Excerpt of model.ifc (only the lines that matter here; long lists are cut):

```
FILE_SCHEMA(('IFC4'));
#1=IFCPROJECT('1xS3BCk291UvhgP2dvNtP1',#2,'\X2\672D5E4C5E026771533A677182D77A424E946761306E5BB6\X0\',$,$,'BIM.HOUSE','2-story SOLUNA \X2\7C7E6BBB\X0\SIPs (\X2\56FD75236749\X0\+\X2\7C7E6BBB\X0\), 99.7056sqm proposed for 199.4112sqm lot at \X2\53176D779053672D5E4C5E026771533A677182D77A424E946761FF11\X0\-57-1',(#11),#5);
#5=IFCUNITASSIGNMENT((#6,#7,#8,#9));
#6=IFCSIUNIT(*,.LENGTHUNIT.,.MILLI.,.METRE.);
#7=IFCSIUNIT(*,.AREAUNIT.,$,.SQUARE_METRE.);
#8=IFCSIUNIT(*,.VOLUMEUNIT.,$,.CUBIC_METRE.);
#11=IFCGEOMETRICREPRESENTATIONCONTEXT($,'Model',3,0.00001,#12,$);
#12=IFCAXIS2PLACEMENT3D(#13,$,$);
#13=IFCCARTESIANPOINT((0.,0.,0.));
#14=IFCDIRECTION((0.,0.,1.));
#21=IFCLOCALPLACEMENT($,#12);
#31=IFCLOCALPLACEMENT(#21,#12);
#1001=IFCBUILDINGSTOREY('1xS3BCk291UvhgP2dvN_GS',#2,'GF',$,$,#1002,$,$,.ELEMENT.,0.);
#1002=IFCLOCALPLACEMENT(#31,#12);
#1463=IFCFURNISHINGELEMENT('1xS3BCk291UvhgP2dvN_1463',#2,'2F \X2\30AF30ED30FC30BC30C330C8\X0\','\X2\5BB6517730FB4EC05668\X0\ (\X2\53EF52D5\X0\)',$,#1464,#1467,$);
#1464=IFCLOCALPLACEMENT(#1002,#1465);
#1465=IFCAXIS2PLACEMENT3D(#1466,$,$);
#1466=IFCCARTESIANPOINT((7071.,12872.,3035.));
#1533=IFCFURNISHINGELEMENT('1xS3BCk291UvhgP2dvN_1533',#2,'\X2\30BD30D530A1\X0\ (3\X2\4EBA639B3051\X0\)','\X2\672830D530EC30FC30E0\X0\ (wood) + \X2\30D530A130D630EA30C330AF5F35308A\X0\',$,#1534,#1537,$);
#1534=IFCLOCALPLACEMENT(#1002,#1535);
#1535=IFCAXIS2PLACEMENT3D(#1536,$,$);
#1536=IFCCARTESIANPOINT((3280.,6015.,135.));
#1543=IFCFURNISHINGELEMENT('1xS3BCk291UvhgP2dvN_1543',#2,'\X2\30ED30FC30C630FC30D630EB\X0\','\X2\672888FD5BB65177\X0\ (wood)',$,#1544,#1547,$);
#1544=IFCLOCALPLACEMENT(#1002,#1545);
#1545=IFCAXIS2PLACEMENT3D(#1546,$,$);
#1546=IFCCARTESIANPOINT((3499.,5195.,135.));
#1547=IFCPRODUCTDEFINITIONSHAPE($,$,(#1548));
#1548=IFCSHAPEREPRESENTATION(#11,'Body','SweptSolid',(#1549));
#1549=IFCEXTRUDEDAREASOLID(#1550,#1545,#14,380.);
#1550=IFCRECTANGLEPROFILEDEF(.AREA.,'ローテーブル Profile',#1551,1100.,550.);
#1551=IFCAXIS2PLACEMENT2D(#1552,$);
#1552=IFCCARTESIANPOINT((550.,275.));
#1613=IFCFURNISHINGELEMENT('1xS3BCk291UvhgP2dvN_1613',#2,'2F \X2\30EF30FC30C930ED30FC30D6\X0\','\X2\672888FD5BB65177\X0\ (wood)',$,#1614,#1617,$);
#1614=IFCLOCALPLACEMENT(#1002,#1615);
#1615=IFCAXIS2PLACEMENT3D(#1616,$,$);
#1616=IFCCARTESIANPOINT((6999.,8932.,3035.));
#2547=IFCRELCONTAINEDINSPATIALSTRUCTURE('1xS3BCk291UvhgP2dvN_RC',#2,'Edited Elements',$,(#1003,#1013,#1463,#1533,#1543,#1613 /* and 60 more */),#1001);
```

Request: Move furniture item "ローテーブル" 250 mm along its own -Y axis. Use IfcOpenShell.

```python
import ifcopenshell
import ifcopenshell.api.geometry
import ifcopenshell.util.placement
import ifcopenshell.util.unit

model = ifcopenshell.open("model.ifc")
unit_scale = ifcopenshell.util.unit.calculate_unit_scale(model)

item = model.by_guid("1xS3BCk291UvhgP2dvN_1543")
matrix = ifcopenshell.util.placement.get_local_placement(item.ObjectPlacement)
matrix[:3, 3] -= matrix[:3, 1] * 0.25 / unit_scale
ifcopenshell.api.geometry.edit_object_placement(model, product=item, matrix=matrix, is_si=False)

print(ifcopenshell.util.placement.get_local_placement(item.ObjectPlacement).round(3) + 0.0)

model.write("model_updated.ifc")
```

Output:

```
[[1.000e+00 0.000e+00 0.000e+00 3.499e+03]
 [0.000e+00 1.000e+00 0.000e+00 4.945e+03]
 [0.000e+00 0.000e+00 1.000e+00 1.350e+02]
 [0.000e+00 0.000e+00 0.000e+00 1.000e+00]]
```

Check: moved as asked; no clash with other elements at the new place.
